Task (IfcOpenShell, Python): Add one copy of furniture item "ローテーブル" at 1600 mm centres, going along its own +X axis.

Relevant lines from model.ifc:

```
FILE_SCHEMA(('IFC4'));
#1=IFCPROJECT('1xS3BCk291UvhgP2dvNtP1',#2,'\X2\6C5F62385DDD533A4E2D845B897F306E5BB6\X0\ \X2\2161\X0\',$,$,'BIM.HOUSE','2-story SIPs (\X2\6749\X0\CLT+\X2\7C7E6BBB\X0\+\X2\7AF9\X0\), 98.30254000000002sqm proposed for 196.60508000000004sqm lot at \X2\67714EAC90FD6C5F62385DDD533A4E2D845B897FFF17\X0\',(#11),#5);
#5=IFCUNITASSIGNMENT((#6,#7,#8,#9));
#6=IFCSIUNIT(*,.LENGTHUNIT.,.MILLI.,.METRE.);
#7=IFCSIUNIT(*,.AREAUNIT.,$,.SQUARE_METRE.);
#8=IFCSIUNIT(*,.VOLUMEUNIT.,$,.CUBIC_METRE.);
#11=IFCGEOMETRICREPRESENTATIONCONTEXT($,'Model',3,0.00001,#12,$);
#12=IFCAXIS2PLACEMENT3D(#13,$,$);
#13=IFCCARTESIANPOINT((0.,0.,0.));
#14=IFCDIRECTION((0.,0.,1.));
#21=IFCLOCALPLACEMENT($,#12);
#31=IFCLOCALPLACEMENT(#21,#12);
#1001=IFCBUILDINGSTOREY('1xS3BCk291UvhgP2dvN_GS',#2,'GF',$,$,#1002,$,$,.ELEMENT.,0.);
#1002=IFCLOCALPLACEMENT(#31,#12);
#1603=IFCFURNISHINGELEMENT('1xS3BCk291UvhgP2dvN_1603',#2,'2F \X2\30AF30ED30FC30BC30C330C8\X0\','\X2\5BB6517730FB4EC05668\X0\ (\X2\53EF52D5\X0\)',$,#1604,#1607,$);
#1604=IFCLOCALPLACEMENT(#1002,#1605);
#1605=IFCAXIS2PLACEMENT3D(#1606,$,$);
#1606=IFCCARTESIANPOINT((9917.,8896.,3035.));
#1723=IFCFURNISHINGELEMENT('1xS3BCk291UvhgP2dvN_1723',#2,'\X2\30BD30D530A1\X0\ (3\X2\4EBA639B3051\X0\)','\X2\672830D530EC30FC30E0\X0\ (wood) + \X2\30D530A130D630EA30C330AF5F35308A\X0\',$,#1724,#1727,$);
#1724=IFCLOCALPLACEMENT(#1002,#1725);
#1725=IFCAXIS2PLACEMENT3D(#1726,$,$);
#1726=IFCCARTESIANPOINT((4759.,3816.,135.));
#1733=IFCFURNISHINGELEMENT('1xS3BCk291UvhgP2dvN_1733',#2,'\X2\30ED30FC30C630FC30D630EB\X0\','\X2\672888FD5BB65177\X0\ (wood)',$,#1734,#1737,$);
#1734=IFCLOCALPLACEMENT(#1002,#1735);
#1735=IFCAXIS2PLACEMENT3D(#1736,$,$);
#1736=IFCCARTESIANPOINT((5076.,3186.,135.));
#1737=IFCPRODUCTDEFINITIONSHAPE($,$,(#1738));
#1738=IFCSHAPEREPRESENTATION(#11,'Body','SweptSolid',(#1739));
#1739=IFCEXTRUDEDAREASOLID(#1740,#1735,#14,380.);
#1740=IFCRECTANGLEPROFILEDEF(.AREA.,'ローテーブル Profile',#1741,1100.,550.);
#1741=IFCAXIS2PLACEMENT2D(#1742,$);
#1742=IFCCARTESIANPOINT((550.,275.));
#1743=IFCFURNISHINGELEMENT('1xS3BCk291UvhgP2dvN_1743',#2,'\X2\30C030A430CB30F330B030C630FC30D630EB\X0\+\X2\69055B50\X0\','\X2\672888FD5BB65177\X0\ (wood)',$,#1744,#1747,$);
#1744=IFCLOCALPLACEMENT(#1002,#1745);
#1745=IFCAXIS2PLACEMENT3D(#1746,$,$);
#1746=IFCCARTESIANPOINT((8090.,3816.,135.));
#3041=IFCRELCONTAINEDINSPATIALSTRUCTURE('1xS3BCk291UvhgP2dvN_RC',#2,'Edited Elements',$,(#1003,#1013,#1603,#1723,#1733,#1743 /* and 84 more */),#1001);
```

```python
import ifcopenshell
import ifcopenshell.api.geometry
import ifcopenshell.api.root
import ifcopenshell.util.element
import ifcopenshell.util.placement
import ifcopenshell.util.unit

model = ifcopenshell.open("model.ifc")
unit_scale = ifcopenshell.util.unit.calculate_unit_scale(model)


def reuse_history(source, copy):
    """copy_class also copies each property set's owner history, people and application; keep the originals."""
    for rel in copy.IsDefinedBy:
        if rel.is_a("IfcRelDefinesByProperties") and (history := rel.RelatingPropertyDefinition.OwnerHistory):
            rel.RelatingPropertyDefinition.OwnerHistory = source.OwnerHistory
            ifcopenshell.util.element.remove_deep2(model, history)


source = model.by_guid("1xS3BCk291UvhgP2dvN_1733")
base = ifcopenshell.util.placement.get_local_placement(source.ObjectPlacement)
step = base[:3, 0] * 1.6 / unit_scale

for i in range(1, 2):
    copy = ifcopenshell.api.root.copy_class(model, product=source)
    copy.Representation = ifcopenshell.util.element.copy_deep(
        model, source.Representation, exclude=["IfcGeometricRepresentationContext", "IfcRepresentationMap"]
    )
    reuse_history(source, copy)
    matrix = base.copy()
    matrix[:3, 3] += i * step
    print("added at", matrix[:3, 3].round(3) + 0.0)
    ifcopenshell.api.geometry.edit_object_placement(model, product=copy, matrix=matrix, is_si=False)

model.write("model_edited.ifc")
```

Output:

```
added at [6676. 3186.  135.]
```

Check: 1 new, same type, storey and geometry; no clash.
